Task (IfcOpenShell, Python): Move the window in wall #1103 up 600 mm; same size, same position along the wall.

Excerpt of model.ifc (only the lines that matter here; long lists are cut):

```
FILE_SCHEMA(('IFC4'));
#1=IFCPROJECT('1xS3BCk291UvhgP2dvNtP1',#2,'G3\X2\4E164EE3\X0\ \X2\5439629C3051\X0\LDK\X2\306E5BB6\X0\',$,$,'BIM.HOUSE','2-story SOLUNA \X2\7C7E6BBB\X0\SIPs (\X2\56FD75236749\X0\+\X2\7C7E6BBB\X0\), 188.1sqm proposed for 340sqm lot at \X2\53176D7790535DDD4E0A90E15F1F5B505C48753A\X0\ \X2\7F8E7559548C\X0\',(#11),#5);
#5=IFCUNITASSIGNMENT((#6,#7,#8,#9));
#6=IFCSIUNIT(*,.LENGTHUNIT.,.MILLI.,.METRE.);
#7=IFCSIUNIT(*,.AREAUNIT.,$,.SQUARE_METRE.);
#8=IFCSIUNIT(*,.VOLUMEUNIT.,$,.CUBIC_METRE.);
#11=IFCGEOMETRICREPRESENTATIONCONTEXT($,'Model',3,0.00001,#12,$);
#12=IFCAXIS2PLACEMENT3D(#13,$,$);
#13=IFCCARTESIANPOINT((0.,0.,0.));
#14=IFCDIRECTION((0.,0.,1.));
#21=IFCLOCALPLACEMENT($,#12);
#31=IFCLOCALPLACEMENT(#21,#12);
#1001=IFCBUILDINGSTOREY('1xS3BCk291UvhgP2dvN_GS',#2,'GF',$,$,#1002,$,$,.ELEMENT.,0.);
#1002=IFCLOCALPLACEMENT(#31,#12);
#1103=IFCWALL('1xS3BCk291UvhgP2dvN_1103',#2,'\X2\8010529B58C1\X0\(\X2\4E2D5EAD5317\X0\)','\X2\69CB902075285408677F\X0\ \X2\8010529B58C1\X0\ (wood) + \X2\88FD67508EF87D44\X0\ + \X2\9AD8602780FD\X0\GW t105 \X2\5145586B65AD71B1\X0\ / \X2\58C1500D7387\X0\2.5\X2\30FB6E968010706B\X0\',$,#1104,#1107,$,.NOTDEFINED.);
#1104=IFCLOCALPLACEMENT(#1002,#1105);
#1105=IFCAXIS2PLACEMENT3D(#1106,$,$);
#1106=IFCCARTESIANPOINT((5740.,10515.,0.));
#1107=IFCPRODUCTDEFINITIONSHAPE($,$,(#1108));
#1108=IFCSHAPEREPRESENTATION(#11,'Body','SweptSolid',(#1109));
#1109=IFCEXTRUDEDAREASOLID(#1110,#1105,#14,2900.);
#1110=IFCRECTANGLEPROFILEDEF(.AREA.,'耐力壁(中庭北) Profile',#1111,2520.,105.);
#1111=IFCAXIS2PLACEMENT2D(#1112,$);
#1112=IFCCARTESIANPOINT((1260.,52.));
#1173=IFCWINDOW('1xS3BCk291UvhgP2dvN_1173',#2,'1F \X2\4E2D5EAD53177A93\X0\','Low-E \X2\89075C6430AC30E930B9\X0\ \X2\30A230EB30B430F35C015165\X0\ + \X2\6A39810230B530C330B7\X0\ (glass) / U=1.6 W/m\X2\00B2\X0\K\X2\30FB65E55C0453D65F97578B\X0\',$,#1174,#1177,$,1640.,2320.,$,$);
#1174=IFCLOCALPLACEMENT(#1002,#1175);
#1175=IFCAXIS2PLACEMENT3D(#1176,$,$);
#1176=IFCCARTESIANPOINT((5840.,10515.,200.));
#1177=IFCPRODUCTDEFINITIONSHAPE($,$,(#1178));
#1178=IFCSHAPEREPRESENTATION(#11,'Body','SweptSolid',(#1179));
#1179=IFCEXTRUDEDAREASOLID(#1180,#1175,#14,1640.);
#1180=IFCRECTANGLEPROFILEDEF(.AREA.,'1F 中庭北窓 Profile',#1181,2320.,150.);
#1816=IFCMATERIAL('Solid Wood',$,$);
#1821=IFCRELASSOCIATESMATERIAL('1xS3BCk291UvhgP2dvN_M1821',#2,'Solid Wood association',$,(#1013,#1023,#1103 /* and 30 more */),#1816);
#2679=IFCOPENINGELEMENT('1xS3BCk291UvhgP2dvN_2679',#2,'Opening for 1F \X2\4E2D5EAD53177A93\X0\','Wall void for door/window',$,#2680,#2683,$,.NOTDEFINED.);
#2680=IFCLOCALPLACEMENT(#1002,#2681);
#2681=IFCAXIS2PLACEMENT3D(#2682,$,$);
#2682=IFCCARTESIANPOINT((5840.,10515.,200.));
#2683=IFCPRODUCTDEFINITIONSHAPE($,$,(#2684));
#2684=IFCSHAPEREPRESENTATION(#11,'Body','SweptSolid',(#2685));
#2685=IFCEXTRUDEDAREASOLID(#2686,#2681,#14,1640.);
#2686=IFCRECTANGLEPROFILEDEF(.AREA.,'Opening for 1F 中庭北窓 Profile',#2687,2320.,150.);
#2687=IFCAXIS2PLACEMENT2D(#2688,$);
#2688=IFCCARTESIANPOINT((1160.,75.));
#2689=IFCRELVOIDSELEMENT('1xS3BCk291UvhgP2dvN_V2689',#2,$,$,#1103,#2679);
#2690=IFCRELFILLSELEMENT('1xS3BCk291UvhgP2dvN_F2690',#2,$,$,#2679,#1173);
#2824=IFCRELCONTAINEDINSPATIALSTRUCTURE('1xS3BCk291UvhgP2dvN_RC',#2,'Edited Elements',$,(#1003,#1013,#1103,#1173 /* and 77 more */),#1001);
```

```python
import numpy as np
import ifcopenshell
import ifcopenshell.api.geometry
import ifcopenshell.util.placement
import ifcopenshell.util.unit

model = ifcopenshell.open("model.ifc")
unit_scale = ifcopenshell.util.unit.calculate_unit_scale(model)

window = model.by_guid("1xS3BCk291UvhgP2dvN_1173")
opening = window.FillsVoids[0].RelatingOpeningElement
dz = 600.0

shift = np.array([0.0, 0.0, dz])
# The window is not placed relative to its opening, so move both.
for product in (opening, window):
    matrix = ifcopenshell.util.placement.get_local_placement(product.ObjectPlacement)
    matrix[:3, 3] += shift
    ifcopenshell.api.geometry.edit_object_placement(model, product=product, matrix=matrix, is_si=False)

print(f"moved by {dz * unit_scale:+.3f} m")

model.write("model_edited.ifc")
```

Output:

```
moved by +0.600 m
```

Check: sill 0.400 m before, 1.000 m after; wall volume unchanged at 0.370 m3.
